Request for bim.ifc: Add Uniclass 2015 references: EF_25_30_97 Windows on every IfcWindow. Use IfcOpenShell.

First a look at what the model holds.

```python
import ifcopenshell

model = ifcopenshell.open("bim.ifc")
print(model.schema)
print("classifications:", [c.Name for c in model.by_type("IfcClassification")])
for ifc_class in ("IfcDoor", "IfcRoof", "IfcStair", "IfcWall", "IfcWindow"):
    print(ifc_class, len(model.by_type(ifc_class)))
```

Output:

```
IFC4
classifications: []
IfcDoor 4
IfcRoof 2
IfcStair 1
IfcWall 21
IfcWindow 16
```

```python
import ifcopenshell
import ifcopenshell.api.classification

model = ifcopenshell.open("bim.ifc")

system = ifcopenshell.api.classification.add_classification(model, classification="Uniclass 2015")

codes = {
    "IfcWindow": ("EF_25_30_97", "Windows"),
}
for ifc_class, (code, name) in codes.items():
    products = model.by_type(ifc_class)
    ifcopenshell.api.classification.add_reference(
        model, products=products, classification=system, identification=code, name=name
    )
    print(code, len(products))

model.write("bim_v2.ifc")
```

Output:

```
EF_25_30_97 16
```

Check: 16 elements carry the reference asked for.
